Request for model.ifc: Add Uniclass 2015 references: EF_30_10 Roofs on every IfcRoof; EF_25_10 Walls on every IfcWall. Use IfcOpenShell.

First a look at what the model holds.

```python
import ifcopenshell

model = ifcopenshell.open("model.ifc")
print(model.schema)
print("classifications:", [c.Name for c in model.by_type("IfcClassification")])
for ifc_class in ("IfcDoor", "IfcRoof", "IfcStair", "IfcWall", "IfcWindow"):
    print(ifc_class, len(model.by_type(ifc_class)))
```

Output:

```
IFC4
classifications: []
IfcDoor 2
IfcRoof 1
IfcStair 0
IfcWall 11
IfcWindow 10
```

```python
import ifcopenshell
import ifcopenshell.api.classification

model = ifcopenshell.open("model.ifc")

system = ifcopenshell.api.classification.add_classification(model, classification="Uniclass 2015")

codes = {
    "IfcRoof": ("EF_30_10", "Roofs"),
    "IfcWall": ("EF_25_10", "Walls"),
}
for ifc_class, (code, name) in codes.items():
    products = model.by_type(ifc_class)
    ifcopenshell.api.classification.add_reference(
        model, products=products, classification=system, identification=code, name=name
    )
    print(code, len(products))

model.write("model_updated.ifc")
```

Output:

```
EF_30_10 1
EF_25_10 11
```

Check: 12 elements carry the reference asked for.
